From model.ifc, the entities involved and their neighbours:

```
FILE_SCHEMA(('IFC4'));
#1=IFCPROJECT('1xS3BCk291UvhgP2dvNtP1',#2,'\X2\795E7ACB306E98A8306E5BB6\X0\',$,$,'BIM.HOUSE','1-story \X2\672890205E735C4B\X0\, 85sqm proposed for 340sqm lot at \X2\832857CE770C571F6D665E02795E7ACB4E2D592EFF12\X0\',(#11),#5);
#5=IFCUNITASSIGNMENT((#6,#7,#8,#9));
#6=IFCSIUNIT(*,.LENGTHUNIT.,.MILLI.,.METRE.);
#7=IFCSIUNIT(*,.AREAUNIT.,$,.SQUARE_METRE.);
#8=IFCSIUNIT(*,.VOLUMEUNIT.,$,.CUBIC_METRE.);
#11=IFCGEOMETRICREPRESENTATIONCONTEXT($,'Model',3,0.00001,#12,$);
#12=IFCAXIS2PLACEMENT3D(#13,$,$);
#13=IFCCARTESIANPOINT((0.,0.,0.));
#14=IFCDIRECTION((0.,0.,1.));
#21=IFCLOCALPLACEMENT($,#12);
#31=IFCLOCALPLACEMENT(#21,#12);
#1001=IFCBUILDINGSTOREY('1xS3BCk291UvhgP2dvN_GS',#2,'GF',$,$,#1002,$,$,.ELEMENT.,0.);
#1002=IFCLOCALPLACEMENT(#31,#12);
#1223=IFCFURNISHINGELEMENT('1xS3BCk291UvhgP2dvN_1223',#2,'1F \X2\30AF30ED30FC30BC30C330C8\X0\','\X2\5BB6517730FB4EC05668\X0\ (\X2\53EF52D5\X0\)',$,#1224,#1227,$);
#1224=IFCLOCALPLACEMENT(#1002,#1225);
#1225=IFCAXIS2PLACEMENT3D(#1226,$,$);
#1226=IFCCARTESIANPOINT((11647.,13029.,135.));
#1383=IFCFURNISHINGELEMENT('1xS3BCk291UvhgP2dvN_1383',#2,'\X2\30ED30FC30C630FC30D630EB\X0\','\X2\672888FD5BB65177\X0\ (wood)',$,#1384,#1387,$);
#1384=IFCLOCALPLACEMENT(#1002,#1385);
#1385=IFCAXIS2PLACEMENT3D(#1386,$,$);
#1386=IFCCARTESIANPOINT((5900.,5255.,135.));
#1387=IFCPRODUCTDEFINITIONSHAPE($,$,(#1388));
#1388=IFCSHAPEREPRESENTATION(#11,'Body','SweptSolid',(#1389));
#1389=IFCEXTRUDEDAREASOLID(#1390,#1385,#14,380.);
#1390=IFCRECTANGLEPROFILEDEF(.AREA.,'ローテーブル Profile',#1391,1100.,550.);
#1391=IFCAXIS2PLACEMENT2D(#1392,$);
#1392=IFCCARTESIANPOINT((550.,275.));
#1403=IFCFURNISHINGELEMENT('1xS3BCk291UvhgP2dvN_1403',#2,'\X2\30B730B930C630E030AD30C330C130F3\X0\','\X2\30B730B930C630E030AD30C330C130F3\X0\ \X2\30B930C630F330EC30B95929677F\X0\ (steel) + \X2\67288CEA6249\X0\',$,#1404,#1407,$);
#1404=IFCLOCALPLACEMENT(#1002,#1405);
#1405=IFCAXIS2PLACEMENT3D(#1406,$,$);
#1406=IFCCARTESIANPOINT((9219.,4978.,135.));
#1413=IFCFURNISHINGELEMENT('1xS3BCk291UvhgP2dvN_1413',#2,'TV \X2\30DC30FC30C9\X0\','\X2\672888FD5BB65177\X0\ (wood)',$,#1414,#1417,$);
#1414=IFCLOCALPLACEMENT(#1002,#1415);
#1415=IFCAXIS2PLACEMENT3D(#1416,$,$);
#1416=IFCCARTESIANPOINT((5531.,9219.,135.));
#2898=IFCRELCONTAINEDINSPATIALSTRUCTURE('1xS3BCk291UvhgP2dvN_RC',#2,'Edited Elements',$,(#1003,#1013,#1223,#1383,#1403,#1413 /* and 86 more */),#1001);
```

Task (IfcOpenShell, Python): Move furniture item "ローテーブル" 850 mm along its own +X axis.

```python
import ifcopenshell
import ifcopenshell.api.geometry
import ifcopenshell.util.placement

model = ifcopenshell.open("model.ifc")

item = model.by_guid("1xS3BCk291UvhgP2dvN_1383")
matrix = ifcopenshell.util.placement.get_local_placement(item.ObjectPlacement)
matrix[:3, 3] += matrix[:3, 0] * 850.0
ifcopenshell.api.geometry.edit_object_placement(model, product=item, matrix=matrix, is_si=False)

print(ifcopenshell.util.placement.get_local_placement(item.ObjectPlacement).round(3) + 0.0)

model.write("model_rev.ifc")
```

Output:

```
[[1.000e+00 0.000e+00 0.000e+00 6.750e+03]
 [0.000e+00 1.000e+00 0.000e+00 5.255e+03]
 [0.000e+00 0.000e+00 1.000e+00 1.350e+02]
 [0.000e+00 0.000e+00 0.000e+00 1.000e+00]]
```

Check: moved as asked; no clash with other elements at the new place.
